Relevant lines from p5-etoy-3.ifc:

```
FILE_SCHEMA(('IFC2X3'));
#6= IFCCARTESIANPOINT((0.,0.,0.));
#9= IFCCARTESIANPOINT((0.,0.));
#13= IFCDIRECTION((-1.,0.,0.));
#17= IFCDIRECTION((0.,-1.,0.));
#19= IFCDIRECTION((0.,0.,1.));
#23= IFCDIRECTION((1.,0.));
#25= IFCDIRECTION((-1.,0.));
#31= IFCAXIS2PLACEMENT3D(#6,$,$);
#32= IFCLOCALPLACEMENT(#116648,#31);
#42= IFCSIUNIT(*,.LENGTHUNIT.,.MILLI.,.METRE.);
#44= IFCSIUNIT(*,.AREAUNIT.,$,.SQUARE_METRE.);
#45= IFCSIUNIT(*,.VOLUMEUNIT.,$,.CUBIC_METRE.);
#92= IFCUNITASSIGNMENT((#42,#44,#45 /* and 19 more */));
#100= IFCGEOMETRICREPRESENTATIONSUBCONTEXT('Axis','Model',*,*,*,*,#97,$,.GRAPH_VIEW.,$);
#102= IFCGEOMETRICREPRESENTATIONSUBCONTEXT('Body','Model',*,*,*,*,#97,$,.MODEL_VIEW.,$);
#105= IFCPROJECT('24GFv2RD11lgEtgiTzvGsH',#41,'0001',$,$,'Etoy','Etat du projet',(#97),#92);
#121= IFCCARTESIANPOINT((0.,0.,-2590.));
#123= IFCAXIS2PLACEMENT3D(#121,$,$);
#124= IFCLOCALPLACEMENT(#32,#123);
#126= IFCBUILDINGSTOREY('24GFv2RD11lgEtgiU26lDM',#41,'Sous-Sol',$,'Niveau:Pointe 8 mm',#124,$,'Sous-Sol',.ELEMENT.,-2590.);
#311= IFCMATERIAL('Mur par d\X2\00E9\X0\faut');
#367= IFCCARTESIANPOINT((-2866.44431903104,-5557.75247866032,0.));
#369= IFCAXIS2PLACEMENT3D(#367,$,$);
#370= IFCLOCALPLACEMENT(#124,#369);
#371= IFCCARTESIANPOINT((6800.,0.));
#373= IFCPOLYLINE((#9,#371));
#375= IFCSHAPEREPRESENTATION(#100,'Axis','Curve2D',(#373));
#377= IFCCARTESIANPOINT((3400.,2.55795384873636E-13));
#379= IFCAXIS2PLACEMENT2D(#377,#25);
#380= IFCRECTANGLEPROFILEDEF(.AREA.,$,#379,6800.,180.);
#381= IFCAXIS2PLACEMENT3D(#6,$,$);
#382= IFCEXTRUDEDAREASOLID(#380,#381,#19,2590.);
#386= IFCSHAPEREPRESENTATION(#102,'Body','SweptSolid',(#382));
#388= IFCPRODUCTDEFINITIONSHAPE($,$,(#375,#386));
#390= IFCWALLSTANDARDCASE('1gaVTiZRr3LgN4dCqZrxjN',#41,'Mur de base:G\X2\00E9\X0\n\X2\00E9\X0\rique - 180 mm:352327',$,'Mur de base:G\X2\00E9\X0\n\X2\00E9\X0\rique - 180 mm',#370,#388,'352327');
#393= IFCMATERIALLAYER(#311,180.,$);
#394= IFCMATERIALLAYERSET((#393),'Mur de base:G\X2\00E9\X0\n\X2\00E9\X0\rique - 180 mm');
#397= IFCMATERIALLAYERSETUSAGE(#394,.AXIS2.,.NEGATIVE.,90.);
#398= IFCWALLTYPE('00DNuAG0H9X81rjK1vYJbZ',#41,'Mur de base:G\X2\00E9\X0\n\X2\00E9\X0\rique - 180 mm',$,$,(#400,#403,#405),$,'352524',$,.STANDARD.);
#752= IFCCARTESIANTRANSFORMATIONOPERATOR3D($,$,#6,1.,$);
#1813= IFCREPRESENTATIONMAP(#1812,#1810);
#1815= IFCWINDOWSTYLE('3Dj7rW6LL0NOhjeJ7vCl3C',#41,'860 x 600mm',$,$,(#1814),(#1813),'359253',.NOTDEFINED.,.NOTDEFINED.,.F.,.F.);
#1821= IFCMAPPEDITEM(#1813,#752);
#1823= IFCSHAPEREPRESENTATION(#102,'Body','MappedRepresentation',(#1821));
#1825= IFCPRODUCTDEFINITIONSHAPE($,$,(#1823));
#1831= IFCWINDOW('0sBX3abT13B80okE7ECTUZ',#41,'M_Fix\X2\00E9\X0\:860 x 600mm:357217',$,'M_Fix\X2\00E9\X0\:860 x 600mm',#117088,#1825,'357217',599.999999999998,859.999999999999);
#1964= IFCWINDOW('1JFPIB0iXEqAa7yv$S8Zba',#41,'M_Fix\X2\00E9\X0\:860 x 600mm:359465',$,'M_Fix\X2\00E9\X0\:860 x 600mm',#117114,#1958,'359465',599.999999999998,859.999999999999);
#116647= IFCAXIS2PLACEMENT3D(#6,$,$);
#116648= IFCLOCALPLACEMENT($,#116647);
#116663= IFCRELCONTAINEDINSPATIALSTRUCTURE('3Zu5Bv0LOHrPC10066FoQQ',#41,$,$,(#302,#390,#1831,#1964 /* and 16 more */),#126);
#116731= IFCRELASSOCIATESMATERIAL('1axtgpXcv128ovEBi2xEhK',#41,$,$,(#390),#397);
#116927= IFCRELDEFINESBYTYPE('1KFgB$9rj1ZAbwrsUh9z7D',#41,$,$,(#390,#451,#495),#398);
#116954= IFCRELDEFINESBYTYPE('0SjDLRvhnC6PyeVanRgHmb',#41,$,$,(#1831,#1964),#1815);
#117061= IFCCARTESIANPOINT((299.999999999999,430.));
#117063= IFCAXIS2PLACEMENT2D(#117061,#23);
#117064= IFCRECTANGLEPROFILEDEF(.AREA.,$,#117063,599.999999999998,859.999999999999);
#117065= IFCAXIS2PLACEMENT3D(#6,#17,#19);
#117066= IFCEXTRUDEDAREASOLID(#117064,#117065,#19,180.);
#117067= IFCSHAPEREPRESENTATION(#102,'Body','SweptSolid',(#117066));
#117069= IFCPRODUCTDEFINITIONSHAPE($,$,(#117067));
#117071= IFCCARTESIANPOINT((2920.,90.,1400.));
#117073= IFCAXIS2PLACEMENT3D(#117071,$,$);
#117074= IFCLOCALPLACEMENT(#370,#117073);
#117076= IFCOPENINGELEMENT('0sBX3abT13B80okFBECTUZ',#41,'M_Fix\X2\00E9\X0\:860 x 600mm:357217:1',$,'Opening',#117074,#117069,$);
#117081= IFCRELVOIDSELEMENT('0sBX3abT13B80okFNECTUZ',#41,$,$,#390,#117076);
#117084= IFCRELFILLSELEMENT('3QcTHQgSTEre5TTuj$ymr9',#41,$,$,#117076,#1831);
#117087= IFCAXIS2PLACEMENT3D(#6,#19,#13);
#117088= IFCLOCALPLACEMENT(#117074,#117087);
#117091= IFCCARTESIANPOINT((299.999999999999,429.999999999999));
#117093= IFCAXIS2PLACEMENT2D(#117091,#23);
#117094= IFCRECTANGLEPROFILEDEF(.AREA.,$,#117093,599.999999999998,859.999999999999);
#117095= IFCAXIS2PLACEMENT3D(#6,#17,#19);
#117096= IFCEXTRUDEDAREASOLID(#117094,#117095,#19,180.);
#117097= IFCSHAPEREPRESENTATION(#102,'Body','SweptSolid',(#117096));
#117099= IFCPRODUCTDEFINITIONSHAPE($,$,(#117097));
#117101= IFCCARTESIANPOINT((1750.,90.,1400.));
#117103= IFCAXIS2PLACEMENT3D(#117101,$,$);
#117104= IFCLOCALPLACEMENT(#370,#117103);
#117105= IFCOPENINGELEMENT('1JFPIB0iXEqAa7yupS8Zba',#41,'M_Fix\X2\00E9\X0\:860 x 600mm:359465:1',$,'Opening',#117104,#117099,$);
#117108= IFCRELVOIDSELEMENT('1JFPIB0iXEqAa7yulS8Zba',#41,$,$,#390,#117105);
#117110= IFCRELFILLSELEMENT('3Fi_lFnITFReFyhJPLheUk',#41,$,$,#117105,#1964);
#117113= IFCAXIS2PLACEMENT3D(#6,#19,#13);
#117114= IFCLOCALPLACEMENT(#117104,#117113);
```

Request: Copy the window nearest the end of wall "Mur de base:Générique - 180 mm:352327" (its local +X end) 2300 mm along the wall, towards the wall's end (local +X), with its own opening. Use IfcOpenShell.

```python
import ifcopenshell
import ifcopenshell.api.feature
import ifcopenshell.api.geometry
import ifcopenshell.api.root
import ifcopenshell.geom
import ifcopenshell.util.element
import ifcopenshell.util.placement
import ifcopenshell.util.shape

model = ifcopenshell.open("p5-etoy-3.ifc")
settings = ifcopenshell.geom.settings()


def volume(element):
    """Net volume in cubic metres, openings subtracted."""
    shape = ifcopenshell.geom.create_shape(settings, element)
    return ifcopenshell.util.shape.get_volume(shape.geometry)


def reuse_history(source, copy):
    """copy_class also copies each property set's owner history, people and application; keep the originals."""
    for rel in copy.IsDefinedBy:
        if rel.is_a("IfcRelDefinesByProperties") and (history := rel.RelatingPropertyDefinition.OwnerHistory):
            rel.RelatingPropertyDefinition.OwnerHistory = source.OwnerHistory
            ifcopenshell.util.element.remove_deep2(model, history)


window = model.by_id(1831)
opening = window.FillsVoids[0].RelatingOpeningElement
wall = opening.VoidsElements[0].RelatingBuildingElement
before = volume(wall)
shift = ifcopenshell.util.placement.get_local_placement(wall.ObjectPlacement)[:3, 0] * 2300.0

# copy_class copies the void relationship, type, container and properties, but no geometry.
new_opening = ifcopenshell.api.root.copy_class(model, product=opening)
new_opening.Representation = ifcopenshell.util.element.copy_deep(
    model, opening.Representation, exclude=["IfcGeometricRepresentationContext", "IfcRepresentationMap"]
)
new_opening.Name = "M_Fixé:860 x 600mm"
new_window = ifcopenshell.api.root.copy_class(model, product=window)
new_window.Representation = ifcopenshell.util.element.copy_deep(
    model, window.Representation, exclude=["IfcGeometricRepresentationContext", "IfcRepresentationMap"]
)
new_window.Name = "M_Fixé:860 x 600mm"
new_window.Tag = None
reuse_history(window, new_window)
fills = ifcopenshell.api.feature.add_filling(model, opening=new_opening, element=new_window)
fills.OwnerHistory = new_window.OwnerHistory  # required in IFC2X3

for old, new in ((opening, new_opening), (window, new_window)):
    matrix = ifcopenshell.util.placement.get_local_placement(old.ObjectPlacement)
    matrix[:3, 3] += shift
    ifcopenshell.api.geometry.edit_object_placement(model, product=new, matrix=matrix, is_si=False)

after = volume(wall)

print(f"wall volume {before:.3f} -> {after:.3f} m3")

model.write("p5-etoy-3_rev.ifc")
```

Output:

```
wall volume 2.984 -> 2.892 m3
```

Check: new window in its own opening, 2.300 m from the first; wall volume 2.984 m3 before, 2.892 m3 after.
